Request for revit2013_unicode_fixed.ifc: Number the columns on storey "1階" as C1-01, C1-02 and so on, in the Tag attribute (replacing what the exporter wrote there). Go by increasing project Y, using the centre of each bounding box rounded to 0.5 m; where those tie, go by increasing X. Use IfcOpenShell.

First a look at what the model holds.

```python
import ifcopenshell
import ifcopenshell.util.element
import ifcopenshell.util.placement

model = ifcopenshell.open("revit2013_unicode_fixed.ifc")
print(model.schema)
storey = next(s for s in model.by_type("IfcBuildingStorey") if s.Name == "1階")
columns = [e for e in ifcopenshell.util.element.get_decomposition(storey) if e.is_a("IfcColumn")]
for e in sorted(columns, key=lambda e: e.id()):
    origin = ifcopenshell.util.placement.get_local_placement(e.ObjectPlacement)[:3, 3]
    print(e.id(), e.Tag, e.Name, origin.round(2) + 0.0, sep=" | ")
```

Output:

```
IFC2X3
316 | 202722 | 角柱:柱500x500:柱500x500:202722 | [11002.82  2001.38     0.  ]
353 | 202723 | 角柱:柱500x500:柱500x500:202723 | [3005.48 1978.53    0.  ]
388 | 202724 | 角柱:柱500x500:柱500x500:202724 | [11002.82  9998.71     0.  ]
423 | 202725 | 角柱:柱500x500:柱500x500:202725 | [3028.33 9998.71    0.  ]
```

```python
import ifcopenshell
import ifcopenshell.geom
import ifcopenshell.util.element
import ifcopenshell.util.shape

model = ifcopenshell.open("revit2013_unicode_fixed.ifc")
settings = ifcopenshell.geom.settings()
settings.set("use-world-coords", True)


def centre(element):
    shape = ifcopenshell.geom.create_shape(settings, element)
    return ifcopenshell.util.shape.get_bbox_centroid(shape.geometry)


storey = next(s for s in model.by_type("IfcBuildingStorey") if s.Name == "1階")
columns = [e for e in ifcopenshell.util.element.get_decomposition(storey) if e.is_a("IfcColumn")]

# Insertion points can sit at a corner or the storey origin, so sort by the geometry (in metres).
centres = {e: centre(e) for e in columns}
columns.sort(key=lambda e: (round(centres[e][1] / 0.5), centres[e][0]))

for i, e in enumerate(columns, start=1):
    number = f"C1-{i:02d}"
    e.Tag = number
    print(e.id(), number)

model.write("revit2013_unicode_fixed_v2.ifc")
```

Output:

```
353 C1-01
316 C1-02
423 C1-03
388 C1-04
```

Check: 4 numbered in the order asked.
